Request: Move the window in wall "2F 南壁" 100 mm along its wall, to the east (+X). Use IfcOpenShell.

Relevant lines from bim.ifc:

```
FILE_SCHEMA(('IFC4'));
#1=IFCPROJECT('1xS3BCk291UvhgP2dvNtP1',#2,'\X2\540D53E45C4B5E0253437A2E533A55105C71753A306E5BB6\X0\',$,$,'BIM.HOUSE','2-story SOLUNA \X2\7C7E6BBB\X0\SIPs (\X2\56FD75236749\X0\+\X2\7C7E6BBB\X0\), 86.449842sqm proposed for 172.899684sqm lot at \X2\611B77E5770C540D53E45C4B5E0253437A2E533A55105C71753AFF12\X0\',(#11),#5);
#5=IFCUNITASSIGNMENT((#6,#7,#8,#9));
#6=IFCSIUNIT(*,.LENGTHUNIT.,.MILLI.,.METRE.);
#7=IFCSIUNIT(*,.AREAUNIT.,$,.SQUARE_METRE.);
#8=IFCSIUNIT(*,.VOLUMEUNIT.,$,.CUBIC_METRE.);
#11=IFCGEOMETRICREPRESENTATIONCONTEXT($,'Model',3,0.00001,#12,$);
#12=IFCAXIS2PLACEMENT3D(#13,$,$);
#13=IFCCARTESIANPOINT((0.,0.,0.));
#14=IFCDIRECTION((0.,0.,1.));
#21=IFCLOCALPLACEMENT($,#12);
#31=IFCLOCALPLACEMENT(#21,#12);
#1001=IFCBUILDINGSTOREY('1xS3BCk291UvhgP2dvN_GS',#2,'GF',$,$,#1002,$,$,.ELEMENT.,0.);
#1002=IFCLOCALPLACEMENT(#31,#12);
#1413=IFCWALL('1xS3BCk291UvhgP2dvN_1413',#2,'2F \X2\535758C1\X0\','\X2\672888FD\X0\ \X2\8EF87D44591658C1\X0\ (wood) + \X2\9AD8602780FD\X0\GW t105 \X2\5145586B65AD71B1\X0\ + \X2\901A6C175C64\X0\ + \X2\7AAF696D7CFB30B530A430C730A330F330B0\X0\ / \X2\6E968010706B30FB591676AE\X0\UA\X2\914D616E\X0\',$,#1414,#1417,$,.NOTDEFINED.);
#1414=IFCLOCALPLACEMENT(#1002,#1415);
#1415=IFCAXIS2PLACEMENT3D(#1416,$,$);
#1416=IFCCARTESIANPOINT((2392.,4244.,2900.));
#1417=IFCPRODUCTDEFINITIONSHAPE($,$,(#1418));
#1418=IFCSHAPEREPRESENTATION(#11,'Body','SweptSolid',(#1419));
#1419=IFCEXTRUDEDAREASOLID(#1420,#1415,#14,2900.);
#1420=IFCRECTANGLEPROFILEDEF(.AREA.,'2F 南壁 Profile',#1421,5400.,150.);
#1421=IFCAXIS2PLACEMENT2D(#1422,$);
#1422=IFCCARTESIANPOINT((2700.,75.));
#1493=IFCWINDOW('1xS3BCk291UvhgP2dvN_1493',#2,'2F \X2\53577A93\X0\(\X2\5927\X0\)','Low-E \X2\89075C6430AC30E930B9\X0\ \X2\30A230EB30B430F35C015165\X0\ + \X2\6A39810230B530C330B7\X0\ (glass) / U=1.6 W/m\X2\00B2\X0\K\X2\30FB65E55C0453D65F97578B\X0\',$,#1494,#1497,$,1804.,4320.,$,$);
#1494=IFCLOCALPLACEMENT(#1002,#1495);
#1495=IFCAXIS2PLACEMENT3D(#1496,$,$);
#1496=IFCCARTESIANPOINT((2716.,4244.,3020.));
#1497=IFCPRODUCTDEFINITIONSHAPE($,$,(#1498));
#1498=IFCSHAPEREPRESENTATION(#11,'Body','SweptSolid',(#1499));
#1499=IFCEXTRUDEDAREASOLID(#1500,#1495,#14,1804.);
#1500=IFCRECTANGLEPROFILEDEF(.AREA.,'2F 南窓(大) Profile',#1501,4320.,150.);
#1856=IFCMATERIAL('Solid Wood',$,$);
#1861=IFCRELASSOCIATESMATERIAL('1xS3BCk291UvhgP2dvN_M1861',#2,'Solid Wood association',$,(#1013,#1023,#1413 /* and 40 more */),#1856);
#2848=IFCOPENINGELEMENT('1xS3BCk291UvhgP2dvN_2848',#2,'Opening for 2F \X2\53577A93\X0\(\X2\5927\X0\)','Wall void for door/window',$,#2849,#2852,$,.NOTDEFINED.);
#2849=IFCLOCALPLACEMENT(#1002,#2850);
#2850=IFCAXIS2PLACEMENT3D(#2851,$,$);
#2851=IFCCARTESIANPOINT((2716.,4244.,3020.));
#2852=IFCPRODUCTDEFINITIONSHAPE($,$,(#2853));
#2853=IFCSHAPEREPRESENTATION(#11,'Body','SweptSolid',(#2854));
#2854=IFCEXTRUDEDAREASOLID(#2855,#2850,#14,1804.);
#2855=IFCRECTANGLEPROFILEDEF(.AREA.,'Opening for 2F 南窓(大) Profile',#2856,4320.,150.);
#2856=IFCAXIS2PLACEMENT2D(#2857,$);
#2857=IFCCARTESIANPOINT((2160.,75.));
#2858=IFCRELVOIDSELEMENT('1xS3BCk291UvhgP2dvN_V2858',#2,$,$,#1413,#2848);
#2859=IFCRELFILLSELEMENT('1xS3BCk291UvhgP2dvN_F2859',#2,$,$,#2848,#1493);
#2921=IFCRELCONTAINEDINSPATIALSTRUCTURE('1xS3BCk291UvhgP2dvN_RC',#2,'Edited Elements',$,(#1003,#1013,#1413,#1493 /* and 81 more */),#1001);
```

```python
import ifcopenshell
import ifcopenshell.api.geometry
import ifcopenshell.util.placement
import ifcopenshell.util.unit

model = ifcopenshell.open("bim.ifc")
unit_scale = ifcopenshell.util.unit.calculate_unit_scale(model)

window = model.by_guid("1xS3BCk291UvhgP2dvN_1493")
opening = window.FillsVoids[0].RelatingOpeningElement
wall = opening.VoidsElements[0].RelatingBuildingElement

wall_matrix = ifcopenshell.util.placement.get_local_placement(wall.ObjectPlacement)
shift = wall_matrix[:3, 0] * 0.1 / unit_scale
before = ifcopenshell.util.placement.get_local_placement(window.ObjectPlacement)[:3, 3].copy()

# The window is not placed relative to its opening, so move both.
for product in (opening, window):
    matrix = ifcopenshell.util.placement.get_local_placement(product.ObjectPlacement)
    matrix[:3, 3] += shift
    ifcopenshell.api.geometry.edit_object_placement(model, product=product, matrix=matrix, is_si=False)

after = ifcopenshell.util.placement.get_local_placement(window.ObjectPlacement)[:3, 3]
print("window moved by", (after - before).round(3) + 0.0)

model.write("bim-out.ifc")
```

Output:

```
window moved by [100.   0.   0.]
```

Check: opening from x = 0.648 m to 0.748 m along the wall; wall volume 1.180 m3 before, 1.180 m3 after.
